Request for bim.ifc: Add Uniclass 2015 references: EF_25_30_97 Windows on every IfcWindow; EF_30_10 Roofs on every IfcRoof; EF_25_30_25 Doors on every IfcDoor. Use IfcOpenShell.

First a look at what the model holds.

```python
import ifcopenshell

model = ifcopenshell.open("bim.ifc")
print(model.schema)
print("classifications:", [c.Name for c in model.by_type("IfcClassification")])
for ifc_class in ("IfcDoor", "IfcRoof", "IfcStair", "IfcWall", "IfcWindow"):
    print(ifc_class, len(model.by_type(ifc_class)))
```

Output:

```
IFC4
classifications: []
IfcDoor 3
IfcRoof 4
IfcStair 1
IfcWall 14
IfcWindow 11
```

```python
import ifcopenshell
import ifcopenshell.api.classification

model = ifcopenshell.open("bim.ifc")

system = ifcopenshell.api.classification.add_classification(model, classification="Uniclass 2015")

codes = {
    "IfcWindow": ("EF_25_30_97", "Windows"),
    "IfcRoof": ("EF_30_10", "Roofs"),
    "IfcDoor": ("EF_25_30_25", "Doors"),
}
for ifc_class, (code, name) in codes.items():
    products = model.by_type(ifc_class)
    ifcopenshell.api.classification.add_reference(
        model, products=products, classification=system, identification=code, name=name
    )
    print(code, len(products))

model.write("bim_v2.ifc")
```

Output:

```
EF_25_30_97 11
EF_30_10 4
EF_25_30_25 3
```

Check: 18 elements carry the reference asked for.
